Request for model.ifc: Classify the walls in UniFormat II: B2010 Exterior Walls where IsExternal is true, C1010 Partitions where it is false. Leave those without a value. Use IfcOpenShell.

First a look at what the model holds.

```python
import ifcopenshell
import ifcopenshell.util.element

model = ifcopenshell.open("model.ifc")
print(model.schema)
print("classifications:", [c.Name for c in model.by_type("IfcClassification")])
values = [ifcopenshell.util.element.get_pset(e, "Pset_WallCommon", "IsExternal") for e in model.by_type("IfcWall")]
for value in (True, False, None):
    print("IsExternal", value, values.count(value))
```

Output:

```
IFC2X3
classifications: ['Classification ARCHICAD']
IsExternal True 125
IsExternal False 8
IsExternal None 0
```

```python
import ifcopenshell
import ifcopenshell.api.classification
import ifcopenshell.util.element

model = ifcopenshell.open("model.ifc")

# IFC2X3 requires Source and Edition and has no link from the project to the system.
system = model.create_entity("IfcClassification", Source="ASTM", Edition="E1557", Name="UniFormat II")

walls = model.by_type("IfcWall")
external = {e: ifcopenshell.util.element.get_pset(e, "Pset_WallCommon", "IsExternal") for e in walls}
for flag, code, name in ((True, "B2010", "Exterior Walls"), (False, "C1010", "Partitions")):
    products = [e for e in walls if external[e] is flag]
    ifcopenshell.api.classification.add_reference(
        model, products=products, classification=system, identification=code, name=name
    )
    print(code, len(products))

model.write("model-out.ifc")
```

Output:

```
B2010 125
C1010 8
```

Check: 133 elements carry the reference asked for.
